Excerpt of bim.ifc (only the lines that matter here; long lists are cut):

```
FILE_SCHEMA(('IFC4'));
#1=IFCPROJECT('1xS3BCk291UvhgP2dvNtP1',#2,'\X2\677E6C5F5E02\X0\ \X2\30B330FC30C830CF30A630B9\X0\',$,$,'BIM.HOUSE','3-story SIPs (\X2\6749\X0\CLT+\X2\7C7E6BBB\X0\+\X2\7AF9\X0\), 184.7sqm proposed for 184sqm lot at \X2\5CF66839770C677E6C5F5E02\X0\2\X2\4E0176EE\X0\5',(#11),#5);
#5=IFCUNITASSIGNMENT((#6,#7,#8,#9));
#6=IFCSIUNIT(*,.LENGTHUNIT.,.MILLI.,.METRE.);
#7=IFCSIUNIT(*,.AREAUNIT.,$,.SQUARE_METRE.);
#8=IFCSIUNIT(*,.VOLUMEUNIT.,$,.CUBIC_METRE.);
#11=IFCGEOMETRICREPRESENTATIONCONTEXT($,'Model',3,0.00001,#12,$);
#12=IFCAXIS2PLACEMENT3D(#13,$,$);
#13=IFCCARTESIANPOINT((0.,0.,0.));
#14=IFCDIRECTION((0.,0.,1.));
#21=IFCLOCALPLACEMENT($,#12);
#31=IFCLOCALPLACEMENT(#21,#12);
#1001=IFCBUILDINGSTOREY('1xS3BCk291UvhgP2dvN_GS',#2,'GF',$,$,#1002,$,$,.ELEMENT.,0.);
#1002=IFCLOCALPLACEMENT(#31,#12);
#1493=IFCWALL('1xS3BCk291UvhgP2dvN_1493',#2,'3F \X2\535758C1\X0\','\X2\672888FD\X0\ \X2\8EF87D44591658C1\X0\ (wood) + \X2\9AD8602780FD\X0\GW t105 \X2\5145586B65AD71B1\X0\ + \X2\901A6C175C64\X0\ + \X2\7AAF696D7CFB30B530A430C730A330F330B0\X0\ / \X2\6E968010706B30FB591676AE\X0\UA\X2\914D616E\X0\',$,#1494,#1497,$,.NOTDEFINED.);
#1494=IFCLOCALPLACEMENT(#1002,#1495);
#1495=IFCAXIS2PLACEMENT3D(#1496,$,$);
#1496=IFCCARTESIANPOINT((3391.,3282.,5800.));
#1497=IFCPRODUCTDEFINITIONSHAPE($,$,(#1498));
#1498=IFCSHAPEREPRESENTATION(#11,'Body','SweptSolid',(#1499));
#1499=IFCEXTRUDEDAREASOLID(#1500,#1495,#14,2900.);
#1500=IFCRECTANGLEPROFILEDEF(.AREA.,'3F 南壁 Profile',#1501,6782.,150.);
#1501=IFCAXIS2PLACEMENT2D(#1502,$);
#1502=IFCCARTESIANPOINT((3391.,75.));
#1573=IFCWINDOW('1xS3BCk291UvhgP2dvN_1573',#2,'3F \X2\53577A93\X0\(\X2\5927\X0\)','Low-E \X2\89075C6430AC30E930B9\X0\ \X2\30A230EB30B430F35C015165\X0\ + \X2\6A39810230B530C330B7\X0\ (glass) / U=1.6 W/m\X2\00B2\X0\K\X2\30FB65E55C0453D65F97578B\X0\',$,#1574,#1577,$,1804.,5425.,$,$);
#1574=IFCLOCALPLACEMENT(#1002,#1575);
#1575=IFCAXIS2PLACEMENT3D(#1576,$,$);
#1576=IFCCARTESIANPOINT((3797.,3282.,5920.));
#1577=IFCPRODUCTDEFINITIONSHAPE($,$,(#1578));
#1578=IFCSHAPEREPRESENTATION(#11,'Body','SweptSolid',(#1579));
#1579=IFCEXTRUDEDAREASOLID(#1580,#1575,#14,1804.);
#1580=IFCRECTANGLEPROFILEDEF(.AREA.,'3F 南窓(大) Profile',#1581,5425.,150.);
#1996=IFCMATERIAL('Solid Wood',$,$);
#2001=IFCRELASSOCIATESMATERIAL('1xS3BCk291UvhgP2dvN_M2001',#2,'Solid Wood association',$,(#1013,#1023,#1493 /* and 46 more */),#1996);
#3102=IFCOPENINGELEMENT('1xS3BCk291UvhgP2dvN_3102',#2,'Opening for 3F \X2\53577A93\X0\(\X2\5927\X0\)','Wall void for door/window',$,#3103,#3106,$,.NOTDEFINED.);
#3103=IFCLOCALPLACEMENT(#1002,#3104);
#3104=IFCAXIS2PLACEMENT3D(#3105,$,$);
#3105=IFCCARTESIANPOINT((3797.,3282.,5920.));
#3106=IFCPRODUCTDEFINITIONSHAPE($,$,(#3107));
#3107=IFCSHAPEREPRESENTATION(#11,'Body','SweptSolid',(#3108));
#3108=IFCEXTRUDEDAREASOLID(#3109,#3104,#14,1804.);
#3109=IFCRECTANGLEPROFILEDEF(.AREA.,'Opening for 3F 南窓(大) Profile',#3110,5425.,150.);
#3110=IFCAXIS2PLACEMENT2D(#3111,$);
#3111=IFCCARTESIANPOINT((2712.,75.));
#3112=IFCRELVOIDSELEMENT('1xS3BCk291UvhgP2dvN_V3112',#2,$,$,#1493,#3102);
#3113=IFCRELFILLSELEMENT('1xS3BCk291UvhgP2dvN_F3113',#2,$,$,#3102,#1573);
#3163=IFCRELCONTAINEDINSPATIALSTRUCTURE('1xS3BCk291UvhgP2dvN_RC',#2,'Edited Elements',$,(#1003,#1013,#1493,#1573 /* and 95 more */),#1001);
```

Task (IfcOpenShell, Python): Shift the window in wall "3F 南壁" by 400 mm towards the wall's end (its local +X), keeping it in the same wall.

```python
import ifcopenshell
import ifcopenshell.api.geometry
import ifcopenshell.util.placement
import ifcopenshell.util.unit

model = ifcopenshell.open("bim.ifc")
unit_scale = ifcopenshell.util.unit.calculate_unit_scale(model)

window = model.by_guid("1xS3BCk291UvhgP2dvN_1573")
opening = window.FillsVoids[0].RelatingOpeningElement
wall = opening.VoidsElements[0].RelatingBuildingElement

wall_matrix = ifcopenshell.util.placement.get_local_placement(wall.ObjectPlacement)
shift = wall_matrix[:3, 0] * 0.4 / unit_scale
before = ifcopenshell.util.placement.get_local_placement(window.ObjectPlacement)[:3, 3].copy()

# The window is not placed relative to its opening, so move both.
for product in (opening, window):
    matrix = ifcopenshell.util.placement.get_local_placement(product.ObjectPlacement)
    matrix[:3, 3] += shift
    ifcopenshell.api.geometry.edit_object_placement(model, product=product, matrix=matrix, is_si=False)

after = ifcopenshell.util.placement.get_local_placement(window.ObjectPlacement)[:3, 3]
print("window moved by", (after - before).round(3) + 0.0)

model.write("bim-out.ifc")
```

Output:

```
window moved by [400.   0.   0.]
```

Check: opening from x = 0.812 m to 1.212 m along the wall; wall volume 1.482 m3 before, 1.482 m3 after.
